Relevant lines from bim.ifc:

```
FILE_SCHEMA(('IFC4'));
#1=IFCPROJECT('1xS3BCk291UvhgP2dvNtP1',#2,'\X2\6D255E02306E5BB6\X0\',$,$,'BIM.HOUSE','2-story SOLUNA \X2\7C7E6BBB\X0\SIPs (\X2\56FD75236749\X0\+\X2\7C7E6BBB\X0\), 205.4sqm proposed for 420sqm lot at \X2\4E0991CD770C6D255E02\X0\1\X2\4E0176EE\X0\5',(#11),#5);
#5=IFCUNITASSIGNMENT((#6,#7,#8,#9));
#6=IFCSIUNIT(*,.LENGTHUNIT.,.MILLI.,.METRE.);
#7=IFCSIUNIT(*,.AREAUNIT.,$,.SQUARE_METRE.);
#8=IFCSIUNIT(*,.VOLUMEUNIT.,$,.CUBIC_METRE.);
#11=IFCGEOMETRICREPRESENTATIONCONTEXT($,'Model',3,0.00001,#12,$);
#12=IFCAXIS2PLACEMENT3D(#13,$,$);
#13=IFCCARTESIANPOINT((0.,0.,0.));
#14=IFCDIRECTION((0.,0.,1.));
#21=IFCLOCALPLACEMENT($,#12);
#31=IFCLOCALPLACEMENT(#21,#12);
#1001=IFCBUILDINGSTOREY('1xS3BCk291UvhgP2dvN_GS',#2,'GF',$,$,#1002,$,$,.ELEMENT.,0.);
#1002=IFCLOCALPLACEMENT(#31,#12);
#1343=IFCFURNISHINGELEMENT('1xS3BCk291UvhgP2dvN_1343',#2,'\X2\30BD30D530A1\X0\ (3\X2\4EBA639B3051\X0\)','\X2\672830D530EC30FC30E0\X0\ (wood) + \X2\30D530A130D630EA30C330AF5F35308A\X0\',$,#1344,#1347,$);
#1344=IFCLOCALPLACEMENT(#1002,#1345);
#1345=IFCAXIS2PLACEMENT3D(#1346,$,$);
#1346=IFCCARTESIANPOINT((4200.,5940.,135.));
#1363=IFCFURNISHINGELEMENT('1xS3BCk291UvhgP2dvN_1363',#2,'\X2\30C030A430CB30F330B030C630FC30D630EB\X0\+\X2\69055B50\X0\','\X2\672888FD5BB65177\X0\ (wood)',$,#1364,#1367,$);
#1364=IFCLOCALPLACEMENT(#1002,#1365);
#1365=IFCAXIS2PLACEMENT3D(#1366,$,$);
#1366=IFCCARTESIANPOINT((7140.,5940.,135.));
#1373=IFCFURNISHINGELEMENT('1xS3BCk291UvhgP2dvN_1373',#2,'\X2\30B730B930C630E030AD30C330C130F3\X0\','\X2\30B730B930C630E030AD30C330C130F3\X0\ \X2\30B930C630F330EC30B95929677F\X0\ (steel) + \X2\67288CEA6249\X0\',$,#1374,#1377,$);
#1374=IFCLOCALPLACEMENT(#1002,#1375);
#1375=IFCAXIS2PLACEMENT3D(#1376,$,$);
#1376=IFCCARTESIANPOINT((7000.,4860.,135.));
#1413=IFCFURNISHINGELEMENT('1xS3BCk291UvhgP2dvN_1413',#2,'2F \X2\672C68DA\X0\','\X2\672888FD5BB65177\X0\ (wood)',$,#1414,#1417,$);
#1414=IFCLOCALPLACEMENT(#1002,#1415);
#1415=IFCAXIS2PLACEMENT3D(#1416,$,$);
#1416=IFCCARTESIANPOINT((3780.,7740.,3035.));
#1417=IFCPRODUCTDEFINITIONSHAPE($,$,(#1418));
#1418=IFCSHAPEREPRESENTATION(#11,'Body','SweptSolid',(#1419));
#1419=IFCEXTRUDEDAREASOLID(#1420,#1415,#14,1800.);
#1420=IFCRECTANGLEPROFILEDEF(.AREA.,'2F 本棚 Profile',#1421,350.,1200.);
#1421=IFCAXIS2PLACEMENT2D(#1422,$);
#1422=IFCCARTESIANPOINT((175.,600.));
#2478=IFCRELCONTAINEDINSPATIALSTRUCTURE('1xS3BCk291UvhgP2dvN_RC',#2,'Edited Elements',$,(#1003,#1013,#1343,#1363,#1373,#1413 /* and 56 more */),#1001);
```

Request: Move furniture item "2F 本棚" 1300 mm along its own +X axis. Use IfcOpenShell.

```python
import ifcopenshell
import ifcopenshell.api.geometry
import ifcopenshell.util.placement

model = ifcopenshell.open("bim.ifc")

item = model.by_guid("1xS3BCk291UvhgP2dvN_1413")
matrix = ifcopenshell.util.placement.get_local_placement(item.ObjectPlacement)
matrix[:3, 3] += matrix[:3, 0] * 1300.0
ifcopenshell.api.geometry.edit_object_placement(model, product=item, matrix=matrix, is_si=False)

print(ifcopenshell.util.placement.get_local_placement(item.ObjectPlacement).round(3) + 0.0)

model.write("bim_edited.ifc")
```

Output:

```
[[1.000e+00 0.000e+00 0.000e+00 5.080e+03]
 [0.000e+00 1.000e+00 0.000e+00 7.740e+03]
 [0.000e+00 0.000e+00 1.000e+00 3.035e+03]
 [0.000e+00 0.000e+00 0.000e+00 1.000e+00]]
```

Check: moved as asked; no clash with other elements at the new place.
